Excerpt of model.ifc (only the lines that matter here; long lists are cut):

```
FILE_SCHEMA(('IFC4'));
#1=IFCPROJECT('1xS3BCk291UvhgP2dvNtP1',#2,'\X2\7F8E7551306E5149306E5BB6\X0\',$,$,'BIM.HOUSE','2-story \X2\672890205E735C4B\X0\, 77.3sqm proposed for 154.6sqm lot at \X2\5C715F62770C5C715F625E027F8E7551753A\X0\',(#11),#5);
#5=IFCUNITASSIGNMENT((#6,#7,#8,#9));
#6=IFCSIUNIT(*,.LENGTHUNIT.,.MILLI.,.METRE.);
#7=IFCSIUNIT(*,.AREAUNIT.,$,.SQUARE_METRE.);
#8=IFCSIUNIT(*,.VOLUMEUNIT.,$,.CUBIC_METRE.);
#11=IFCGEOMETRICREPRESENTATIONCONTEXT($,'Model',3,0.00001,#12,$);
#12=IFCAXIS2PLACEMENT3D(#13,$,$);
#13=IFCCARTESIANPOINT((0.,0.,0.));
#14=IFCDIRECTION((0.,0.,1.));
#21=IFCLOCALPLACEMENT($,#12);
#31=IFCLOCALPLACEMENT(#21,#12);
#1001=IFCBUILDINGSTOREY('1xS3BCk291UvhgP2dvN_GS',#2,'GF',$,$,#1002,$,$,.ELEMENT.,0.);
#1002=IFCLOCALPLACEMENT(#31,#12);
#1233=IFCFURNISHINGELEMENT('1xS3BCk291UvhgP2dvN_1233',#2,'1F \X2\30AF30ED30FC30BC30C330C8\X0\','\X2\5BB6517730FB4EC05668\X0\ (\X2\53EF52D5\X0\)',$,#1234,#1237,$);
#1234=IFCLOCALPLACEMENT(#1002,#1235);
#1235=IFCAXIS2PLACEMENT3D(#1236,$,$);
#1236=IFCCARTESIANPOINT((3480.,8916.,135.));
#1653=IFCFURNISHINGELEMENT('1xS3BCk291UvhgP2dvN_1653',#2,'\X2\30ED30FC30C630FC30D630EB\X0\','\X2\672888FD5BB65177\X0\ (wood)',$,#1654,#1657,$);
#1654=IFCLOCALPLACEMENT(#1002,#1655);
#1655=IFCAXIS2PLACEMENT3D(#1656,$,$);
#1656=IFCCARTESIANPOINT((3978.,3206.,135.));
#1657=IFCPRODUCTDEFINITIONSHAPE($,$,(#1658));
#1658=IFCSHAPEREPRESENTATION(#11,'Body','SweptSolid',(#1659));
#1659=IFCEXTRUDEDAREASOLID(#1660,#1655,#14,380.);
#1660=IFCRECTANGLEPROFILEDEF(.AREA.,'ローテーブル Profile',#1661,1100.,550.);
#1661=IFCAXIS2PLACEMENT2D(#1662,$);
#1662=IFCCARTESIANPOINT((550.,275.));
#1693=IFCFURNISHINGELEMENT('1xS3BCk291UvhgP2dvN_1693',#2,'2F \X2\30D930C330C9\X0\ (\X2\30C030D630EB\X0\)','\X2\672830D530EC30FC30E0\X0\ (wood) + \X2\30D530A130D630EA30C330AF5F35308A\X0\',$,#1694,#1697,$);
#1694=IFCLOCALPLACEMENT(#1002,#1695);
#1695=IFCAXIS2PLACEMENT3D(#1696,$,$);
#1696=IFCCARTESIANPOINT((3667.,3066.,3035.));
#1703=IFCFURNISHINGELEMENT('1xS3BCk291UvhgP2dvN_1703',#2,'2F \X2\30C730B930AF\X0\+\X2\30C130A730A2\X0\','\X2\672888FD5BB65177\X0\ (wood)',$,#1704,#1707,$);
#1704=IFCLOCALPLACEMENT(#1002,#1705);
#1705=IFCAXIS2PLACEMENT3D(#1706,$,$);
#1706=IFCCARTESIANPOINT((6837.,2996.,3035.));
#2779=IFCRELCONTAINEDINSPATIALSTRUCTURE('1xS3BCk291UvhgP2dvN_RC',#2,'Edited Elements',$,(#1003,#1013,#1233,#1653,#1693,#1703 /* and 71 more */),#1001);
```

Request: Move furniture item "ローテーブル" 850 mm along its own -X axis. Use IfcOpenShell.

```python
import ifcopenshell
import ifcopenshell.api.geometry
import ifcopenshell.util.placement

model = ifcopenshell.open("model.ifc")

item = model.by_id(1653)
matrix = ifcopenshell.util.placement.get_local_placement(item.ObjectPlacement)
matrix[:3, 3] -= matrix[:3, 0] * 850.0
ifcopenshell.api.geometry.edit_object_placement(model, product=item, matrix=matrix, is_si=False)

print(ifcopenshell.util.placement.get_local_placement(item.ObjectPlacement).round(3) + 0.0)

model.write("model_rev.ifc")
```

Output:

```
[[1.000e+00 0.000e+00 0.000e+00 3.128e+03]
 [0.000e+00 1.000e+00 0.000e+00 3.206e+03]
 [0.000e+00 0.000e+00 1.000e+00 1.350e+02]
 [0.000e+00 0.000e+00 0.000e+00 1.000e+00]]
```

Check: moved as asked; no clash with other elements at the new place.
